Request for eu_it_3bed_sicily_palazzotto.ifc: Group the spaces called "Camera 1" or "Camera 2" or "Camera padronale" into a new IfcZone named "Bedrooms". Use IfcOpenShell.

First a look at what the model holds.

```python
import ifcopenshell

model = ifcopenshell.open("eu_it_3bed_sicily_palazzotto.ifc")
print(model.schema)
seen = {}
for space in model.by_type("IfcSpace"):
    seen[space.LongName] = seen.get(space.LongName, 0) + 1
for name, count in sorted(seen.items(), key=str):
    print(count, "x", name)
print("zones:", [z.Name for z in model.by_type("IfcZone")][:20])
```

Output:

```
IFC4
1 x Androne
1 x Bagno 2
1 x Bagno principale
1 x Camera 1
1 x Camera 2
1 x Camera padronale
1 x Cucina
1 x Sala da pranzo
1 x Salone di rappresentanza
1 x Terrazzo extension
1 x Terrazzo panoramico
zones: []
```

```python
import ifcopenshell
import ifcopenshell.api.group
import ifcopenshell.api.root

model = ifcopenshell.open("eu_it_3bed_sicily_palazzotto.ifc")

names = {"Camera 1", "Camera 2", "Camera padronale"}
spaces = [s for s in model.by_type("IfcSpace") if s.LongName in names]

zone = ifcopenshell.api.root.create_entity(model, ifc_class="IfcZone", name="Bedrooms")
ifcopenshell.api.group.assign_group(model, products=spaces, group=zone)
print(len(spaces), "spaces in", zone.Name)

model.write("eu_it_3bed_sicily_palazzotto_v2.ifc")
```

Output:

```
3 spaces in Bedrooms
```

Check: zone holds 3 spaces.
